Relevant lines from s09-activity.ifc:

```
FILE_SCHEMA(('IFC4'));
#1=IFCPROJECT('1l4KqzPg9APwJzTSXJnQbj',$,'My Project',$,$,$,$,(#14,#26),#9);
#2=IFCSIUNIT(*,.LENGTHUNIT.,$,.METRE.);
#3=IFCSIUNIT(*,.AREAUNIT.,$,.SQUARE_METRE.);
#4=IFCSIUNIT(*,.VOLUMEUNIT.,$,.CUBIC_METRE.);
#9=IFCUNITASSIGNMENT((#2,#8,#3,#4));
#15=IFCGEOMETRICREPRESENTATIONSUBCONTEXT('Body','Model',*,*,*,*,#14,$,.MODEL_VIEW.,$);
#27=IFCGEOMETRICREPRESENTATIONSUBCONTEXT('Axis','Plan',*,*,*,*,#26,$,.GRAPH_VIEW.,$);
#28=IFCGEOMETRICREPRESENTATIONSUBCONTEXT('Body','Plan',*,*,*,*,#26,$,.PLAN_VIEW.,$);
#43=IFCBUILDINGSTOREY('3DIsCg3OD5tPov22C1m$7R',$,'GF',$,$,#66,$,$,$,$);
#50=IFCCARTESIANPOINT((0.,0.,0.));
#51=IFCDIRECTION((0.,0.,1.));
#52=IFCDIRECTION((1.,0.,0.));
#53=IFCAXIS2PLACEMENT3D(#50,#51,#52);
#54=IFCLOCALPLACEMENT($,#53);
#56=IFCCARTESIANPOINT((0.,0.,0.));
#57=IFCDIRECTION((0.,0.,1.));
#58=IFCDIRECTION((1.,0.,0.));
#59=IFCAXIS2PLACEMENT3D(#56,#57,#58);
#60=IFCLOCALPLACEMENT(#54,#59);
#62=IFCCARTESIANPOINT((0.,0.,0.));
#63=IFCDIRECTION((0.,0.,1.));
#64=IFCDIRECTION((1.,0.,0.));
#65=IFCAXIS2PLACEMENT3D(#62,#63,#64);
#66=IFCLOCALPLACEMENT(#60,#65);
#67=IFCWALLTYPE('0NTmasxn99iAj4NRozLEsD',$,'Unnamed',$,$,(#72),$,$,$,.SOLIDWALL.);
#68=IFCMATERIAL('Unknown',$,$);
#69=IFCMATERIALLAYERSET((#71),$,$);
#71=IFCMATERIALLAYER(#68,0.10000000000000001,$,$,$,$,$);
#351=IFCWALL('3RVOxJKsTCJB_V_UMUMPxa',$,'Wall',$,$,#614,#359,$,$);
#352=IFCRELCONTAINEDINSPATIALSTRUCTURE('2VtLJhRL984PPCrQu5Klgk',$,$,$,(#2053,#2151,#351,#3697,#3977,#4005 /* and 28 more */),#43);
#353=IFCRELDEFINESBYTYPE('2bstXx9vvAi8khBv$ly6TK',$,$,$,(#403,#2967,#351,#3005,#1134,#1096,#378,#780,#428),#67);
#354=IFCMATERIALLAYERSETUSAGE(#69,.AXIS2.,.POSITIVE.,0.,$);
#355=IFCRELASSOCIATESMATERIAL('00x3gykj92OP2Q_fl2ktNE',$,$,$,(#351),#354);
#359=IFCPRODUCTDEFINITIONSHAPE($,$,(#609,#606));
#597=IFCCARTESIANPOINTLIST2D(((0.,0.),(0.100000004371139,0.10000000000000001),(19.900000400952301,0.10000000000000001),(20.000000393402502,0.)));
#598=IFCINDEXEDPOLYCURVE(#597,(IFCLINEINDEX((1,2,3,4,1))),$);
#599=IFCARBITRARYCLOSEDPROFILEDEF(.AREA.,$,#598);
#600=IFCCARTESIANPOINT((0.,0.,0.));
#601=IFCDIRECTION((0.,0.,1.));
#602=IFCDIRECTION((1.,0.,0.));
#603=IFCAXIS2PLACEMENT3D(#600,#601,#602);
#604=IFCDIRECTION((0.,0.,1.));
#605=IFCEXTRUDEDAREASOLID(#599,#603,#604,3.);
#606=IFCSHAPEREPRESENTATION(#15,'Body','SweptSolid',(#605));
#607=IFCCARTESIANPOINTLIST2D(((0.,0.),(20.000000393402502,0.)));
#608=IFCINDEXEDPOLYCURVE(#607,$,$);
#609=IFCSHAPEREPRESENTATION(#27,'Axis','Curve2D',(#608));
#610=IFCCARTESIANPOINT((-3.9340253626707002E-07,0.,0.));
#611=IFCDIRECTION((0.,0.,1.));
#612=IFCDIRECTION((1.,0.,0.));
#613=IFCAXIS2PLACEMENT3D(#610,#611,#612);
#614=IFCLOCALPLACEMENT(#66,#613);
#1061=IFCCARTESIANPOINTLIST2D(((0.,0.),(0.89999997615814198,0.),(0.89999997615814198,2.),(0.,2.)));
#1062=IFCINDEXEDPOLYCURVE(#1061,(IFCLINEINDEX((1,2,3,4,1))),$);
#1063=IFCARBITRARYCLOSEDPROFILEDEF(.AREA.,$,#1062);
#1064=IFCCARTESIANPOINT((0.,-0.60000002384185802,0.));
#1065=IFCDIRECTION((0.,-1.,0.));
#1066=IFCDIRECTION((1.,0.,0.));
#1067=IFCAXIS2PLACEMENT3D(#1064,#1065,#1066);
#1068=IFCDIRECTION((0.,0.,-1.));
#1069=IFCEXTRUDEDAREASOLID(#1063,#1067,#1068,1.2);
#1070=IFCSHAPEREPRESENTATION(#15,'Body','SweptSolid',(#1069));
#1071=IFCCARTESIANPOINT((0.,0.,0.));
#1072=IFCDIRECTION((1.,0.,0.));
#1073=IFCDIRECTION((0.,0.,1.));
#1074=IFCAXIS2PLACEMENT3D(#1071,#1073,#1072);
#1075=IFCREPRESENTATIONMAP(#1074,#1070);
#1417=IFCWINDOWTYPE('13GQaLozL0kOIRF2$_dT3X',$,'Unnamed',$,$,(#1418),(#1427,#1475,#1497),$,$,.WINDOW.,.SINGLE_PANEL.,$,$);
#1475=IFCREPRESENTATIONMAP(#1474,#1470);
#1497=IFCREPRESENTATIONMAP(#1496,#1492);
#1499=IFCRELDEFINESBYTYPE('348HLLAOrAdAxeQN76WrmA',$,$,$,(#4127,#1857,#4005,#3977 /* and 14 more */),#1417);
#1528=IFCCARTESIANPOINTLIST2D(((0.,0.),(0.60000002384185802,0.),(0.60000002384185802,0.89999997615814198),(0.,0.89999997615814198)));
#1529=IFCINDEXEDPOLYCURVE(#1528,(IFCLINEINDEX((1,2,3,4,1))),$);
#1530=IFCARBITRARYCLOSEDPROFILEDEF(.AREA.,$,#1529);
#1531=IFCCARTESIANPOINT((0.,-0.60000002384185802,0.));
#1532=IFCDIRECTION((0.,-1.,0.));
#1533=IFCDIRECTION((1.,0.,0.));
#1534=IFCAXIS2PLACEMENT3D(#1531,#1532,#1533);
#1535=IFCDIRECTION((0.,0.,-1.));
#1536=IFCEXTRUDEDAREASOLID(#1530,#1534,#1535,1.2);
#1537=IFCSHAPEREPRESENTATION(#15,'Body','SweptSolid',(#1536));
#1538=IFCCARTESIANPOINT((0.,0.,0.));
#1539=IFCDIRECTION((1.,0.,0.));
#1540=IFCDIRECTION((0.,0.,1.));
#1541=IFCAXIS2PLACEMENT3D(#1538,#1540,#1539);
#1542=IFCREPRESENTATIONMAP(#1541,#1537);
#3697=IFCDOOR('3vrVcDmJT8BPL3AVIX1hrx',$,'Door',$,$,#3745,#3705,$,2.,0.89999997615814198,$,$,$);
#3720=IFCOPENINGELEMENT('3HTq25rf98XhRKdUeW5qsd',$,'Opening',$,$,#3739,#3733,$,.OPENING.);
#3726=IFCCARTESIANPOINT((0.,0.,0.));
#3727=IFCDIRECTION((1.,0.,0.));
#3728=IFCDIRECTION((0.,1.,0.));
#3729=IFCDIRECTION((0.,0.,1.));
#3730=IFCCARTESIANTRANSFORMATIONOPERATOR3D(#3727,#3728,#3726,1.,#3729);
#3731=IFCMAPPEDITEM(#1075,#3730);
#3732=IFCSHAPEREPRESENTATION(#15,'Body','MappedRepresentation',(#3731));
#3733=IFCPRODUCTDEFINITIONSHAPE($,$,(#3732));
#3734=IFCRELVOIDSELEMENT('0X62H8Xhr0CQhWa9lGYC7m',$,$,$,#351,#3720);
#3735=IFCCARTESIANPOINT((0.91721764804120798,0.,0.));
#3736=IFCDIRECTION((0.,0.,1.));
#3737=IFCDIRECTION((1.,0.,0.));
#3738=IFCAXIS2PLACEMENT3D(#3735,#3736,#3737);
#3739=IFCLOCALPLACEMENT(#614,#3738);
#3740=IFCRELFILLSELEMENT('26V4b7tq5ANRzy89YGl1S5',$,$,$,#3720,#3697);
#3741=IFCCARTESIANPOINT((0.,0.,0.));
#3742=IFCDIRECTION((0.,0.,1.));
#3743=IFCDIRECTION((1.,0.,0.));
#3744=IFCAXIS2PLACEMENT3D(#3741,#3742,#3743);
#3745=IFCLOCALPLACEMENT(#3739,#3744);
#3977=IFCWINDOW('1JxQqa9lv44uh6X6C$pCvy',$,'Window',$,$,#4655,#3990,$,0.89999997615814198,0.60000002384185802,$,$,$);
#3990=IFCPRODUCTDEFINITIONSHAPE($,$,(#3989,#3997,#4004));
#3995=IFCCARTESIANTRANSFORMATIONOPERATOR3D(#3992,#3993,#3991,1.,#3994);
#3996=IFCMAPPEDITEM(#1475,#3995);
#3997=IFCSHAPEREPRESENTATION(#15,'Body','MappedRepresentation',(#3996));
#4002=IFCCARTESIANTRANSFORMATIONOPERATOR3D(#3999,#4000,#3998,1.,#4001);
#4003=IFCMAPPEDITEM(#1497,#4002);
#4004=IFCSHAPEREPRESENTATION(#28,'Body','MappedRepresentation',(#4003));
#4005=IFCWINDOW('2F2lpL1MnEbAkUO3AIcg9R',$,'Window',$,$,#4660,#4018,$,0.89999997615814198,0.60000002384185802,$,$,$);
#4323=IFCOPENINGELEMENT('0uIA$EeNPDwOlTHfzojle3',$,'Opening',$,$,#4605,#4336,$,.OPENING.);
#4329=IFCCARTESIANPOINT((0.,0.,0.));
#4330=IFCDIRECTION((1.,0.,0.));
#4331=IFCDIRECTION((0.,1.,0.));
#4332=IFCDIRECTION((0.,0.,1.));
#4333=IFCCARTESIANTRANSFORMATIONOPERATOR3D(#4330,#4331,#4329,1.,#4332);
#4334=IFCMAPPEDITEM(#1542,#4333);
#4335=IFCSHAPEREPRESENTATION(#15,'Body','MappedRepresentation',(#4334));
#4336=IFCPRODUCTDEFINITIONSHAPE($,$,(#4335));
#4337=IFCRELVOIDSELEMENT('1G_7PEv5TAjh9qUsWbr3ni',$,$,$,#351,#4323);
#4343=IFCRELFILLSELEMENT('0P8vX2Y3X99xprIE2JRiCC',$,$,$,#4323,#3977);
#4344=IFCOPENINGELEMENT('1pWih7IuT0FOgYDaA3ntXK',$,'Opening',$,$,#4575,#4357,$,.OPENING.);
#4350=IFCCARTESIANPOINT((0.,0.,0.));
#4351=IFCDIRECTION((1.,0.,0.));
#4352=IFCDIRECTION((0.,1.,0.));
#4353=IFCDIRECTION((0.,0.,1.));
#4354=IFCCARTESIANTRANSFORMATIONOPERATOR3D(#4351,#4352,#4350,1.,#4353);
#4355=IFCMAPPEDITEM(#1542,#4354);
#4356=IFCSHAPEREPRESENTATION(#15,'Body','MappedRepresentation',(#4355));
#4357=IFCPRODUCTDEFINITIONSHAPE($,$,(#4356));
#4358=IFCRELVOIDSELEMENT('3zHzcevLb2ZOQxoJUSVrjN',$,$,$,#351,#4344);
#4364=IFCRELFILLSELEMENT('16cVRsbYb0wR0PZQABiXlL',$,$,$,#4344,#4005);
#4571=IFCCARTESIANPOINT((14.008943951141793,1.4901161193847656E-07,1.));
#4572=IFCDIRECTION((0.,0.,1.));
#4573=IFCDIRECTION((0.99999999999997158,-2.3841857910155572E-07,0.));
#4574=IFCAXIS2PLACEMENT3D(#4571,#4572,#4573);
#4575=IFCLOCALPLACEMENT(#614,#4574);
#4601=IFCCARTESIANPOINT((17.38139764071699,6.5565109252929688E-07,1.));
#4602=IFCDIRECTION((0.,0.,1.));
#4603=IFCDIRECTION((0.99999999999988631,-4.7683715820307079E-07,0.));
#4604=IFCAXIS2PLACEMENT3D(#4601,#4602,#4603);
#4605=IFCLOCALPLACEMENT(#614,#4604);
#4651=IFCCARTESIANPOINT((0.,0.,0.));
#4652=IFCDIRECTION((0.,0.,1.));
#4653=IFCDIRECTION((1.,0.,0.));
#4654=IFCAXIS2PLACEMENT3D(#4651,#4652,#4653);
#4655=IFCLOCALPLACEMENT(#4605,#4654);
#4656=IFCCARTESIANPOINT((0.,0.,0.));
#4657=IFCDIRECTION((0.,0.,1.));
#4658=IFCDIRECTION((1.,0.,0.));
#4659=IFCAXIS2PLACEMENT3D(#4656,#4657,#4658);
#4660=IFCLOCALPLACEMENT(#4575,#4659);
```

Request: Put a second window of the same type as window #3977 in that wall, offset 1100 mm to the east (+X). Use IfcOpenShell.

```python
import ifcopenshell
import ifcopenshell.api.feature
import ifcopenshell.api.geometry
import ifcopenshell.api.root
import ifcopenshell.geom
import ifcopenshell.util.element
import ifcopenshell.util.placement
import ifcopenshell.util.shape
import ifcopenshell.util.unit

model = ifcopenshell.open("s09-activity.ifc")
unit_scale = ifcopenshell.util.unit.calculate_unit_scale(model)
settings = ifcopenshell.geom.settings()


def volume(element):
    """Net volume in cubic metres, openings subtracted."""
    shape = ifcopenshell.geom.create_shape(settings, element)
    return ifcopenshell.util.shape.get_volume(shape.geometry)


window = model.by_guid("1JxQqa9lv44uh6X6C$pCvy")
opening = window.FillsVoids[0].RelatingOpeningElement
wall = opening.VoidsElements[0].RelatingBuildingElement
before = volume(wall)
shift = ifcopenshell.util.placement.get_local_placement(wall.ObjectPlacement)[:3, 0] * 1.1 / unit_scale

# copy_class copies the void relationship, type, container and properties, but no geometry.
new_opening = ifcopenshell.api.root.copy_class(model, product=opening)
new_opening.Representation = ifcopenshell.util.element.copy_deep(
    model, opening.Representation, exclude=["IfcGeometricRepresentationContext", "IfcRepresentationMap"]
)
new_window = ifcopenshell.api.root.copy_class(model, product=window)
new_window.Representation = ifcopenshell.util.element.copy_deep(
    model, window.Representation, exclude=["IfcGeometricRepresentationContext", "IfcRepresentationMap"]
)
ifcopenshell.api.feature.add_filling(model, opening=new_opening, element=new_window)

for old, new in ((opening, new_opening), (window, new_window)):
    matrix = ifcopenshell.util.placement.get_local_placement(old.ObjectPlacement)
    matrix[:3, 3] += shift
    ifcopenshell.api.geometry.edit_object_placement(model, product=new, matrix=matrix, is_si=False)

after = volume(wall)

print(f"wall volume {before:.3f} -> {after:.3f} m3")

model.write("s09-activity-out.ifc")
```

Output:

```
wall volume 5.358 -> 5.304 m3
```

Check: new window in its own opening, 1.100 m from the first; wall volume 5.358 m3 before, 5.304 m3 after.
